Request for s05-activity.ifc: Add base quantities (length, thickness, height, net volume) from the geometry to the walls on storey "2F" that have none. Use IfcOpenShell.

First a look at what the model holds.

```python
import ifcopenshell
import ifcopenshell.util.element
import ifcopenshell.util.unit

model = ifcopenshell.open("s05-activity.ifc")
print(model.schema)
for unit_type in ("LENGTHUNIT", "AREAUNIT", "VOLUMEUNIT"):
    print(unit_type, ifcopenshell.util.unit.calculate_unit_scale(model, unit_type))
storey = next(s for s in model.by_type("IfcBuildingStorey") if s.Name == "2F")
walls = [e for e in ifcopenshell.util.element.get_decomposition(storey) if e.is_a("IfcWall")]
for e in sorted(walls, key=lambda e: e.id()):
    print(e.id(), e.is_a(), e.Name, list(ifcopenshell.util.element.get_psets(e, qtos_only=True)), sep=" | ")
```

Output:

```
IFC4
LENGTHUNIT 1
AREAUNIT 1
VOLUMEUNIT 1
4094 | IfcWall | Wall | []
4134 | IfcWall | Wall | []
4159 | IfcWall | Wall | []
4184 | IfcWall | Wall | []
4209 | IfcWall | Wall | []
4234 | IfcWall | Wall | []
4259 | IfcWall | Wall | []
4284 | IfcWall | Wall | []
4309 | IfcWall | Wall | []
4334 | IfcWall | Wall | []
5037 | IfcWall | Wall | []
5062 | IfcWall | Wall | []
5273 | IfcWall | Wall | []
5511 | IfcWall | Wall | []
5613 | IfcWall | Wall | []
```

```python
import ifcopenshell
import ifcopenshell.api.pset
import ifcopenshell.geom
import ifcopenshell.util.element
import ifcopenshell.util.shape
import ifcopenshell.util.unit

model = ifcopenshell.open("s05-activity.ifc")
unit_scale = ifcopenshell.util.unit.calculate_unit_scale(model)
volume_scale = ifcopenshell.util.unit.calculate_unit_scale(model, "VOLUMEUNIT")
settings = ifcopenshell.geom.settings()

storey = next(s for s in model.by_type("IfcBuildingStorey") if s.Name == "2F")
walls = [e for e in ifcopenshell.util.element.get_decomposition(storey) if e.is_a("IfcWall")]

for e in sorted(walls, key=lambda e: e.id()):
    if ifcopenshell.util.element.get_psets(e, qtos_only=True, should_inherit=False):
        continue
    # Geometry comes back in metres, in the element's own axes.
    shape = ifcopenshell.geom.create_shape(settings, e)
    values = {
        "Length": ifcopenshell.util.shape.get_x(shape.geometry) / unit_scale,
        "Width": ifcopenshell.util.shape.get_y(shape.geometry) / unit_scale,
        "Height": ifcopenshell.util.shape.get_z(shape.geometry) / unit_scale,
        "NetVolume": ifcopenshell.util.shape.get_volume(shape.geometry) / volume_scale,
    }
    qto = ifcopenshell.api.pset.add_qto(model, product=e, name="Qto_WallBaseQuantities")
    ifcopenshell.api.pset.edit_qto(model, qto=qto, properties=values)
    print(e.id(), {k: round(v, 3) for k, v in values.items()})

model.write("s05-activity_v2.ifc")
```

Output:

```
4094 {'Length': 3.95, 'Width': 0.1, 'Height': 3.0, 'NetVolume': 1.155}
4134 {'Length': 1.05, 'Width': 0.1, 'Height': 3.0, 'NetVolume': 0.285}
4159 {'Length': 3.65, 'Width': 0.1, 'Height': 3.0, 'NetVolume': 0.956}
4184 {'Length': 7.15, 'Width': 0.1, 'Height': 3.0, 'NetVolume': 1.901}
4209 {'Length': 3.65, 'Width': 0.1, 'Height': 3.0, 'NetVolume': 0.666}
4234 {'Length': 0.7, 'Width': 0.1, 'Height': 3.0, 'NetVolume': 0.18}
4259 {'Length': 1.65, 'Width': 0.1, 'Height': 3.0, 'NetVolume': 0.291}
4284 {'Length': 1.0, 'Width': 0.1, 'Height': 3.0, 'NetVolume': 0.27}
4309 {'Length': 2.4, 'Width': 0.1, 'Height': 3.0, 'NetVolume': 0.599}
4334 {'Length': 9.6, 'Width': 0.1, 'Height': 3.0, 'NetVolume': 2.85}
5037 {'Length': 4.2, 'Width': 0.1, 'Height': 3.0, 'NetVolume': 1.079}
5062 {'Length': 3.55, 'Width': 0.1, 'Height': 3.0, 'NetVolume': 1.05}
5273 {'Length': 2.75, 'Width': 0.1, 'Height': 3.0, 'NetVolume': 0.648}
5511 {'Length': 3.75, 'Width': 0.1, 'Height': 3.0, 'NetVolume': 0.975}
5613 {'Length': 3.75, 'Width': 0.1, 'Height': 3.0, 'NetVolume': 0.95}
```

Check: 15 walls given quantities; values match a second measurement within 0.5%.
